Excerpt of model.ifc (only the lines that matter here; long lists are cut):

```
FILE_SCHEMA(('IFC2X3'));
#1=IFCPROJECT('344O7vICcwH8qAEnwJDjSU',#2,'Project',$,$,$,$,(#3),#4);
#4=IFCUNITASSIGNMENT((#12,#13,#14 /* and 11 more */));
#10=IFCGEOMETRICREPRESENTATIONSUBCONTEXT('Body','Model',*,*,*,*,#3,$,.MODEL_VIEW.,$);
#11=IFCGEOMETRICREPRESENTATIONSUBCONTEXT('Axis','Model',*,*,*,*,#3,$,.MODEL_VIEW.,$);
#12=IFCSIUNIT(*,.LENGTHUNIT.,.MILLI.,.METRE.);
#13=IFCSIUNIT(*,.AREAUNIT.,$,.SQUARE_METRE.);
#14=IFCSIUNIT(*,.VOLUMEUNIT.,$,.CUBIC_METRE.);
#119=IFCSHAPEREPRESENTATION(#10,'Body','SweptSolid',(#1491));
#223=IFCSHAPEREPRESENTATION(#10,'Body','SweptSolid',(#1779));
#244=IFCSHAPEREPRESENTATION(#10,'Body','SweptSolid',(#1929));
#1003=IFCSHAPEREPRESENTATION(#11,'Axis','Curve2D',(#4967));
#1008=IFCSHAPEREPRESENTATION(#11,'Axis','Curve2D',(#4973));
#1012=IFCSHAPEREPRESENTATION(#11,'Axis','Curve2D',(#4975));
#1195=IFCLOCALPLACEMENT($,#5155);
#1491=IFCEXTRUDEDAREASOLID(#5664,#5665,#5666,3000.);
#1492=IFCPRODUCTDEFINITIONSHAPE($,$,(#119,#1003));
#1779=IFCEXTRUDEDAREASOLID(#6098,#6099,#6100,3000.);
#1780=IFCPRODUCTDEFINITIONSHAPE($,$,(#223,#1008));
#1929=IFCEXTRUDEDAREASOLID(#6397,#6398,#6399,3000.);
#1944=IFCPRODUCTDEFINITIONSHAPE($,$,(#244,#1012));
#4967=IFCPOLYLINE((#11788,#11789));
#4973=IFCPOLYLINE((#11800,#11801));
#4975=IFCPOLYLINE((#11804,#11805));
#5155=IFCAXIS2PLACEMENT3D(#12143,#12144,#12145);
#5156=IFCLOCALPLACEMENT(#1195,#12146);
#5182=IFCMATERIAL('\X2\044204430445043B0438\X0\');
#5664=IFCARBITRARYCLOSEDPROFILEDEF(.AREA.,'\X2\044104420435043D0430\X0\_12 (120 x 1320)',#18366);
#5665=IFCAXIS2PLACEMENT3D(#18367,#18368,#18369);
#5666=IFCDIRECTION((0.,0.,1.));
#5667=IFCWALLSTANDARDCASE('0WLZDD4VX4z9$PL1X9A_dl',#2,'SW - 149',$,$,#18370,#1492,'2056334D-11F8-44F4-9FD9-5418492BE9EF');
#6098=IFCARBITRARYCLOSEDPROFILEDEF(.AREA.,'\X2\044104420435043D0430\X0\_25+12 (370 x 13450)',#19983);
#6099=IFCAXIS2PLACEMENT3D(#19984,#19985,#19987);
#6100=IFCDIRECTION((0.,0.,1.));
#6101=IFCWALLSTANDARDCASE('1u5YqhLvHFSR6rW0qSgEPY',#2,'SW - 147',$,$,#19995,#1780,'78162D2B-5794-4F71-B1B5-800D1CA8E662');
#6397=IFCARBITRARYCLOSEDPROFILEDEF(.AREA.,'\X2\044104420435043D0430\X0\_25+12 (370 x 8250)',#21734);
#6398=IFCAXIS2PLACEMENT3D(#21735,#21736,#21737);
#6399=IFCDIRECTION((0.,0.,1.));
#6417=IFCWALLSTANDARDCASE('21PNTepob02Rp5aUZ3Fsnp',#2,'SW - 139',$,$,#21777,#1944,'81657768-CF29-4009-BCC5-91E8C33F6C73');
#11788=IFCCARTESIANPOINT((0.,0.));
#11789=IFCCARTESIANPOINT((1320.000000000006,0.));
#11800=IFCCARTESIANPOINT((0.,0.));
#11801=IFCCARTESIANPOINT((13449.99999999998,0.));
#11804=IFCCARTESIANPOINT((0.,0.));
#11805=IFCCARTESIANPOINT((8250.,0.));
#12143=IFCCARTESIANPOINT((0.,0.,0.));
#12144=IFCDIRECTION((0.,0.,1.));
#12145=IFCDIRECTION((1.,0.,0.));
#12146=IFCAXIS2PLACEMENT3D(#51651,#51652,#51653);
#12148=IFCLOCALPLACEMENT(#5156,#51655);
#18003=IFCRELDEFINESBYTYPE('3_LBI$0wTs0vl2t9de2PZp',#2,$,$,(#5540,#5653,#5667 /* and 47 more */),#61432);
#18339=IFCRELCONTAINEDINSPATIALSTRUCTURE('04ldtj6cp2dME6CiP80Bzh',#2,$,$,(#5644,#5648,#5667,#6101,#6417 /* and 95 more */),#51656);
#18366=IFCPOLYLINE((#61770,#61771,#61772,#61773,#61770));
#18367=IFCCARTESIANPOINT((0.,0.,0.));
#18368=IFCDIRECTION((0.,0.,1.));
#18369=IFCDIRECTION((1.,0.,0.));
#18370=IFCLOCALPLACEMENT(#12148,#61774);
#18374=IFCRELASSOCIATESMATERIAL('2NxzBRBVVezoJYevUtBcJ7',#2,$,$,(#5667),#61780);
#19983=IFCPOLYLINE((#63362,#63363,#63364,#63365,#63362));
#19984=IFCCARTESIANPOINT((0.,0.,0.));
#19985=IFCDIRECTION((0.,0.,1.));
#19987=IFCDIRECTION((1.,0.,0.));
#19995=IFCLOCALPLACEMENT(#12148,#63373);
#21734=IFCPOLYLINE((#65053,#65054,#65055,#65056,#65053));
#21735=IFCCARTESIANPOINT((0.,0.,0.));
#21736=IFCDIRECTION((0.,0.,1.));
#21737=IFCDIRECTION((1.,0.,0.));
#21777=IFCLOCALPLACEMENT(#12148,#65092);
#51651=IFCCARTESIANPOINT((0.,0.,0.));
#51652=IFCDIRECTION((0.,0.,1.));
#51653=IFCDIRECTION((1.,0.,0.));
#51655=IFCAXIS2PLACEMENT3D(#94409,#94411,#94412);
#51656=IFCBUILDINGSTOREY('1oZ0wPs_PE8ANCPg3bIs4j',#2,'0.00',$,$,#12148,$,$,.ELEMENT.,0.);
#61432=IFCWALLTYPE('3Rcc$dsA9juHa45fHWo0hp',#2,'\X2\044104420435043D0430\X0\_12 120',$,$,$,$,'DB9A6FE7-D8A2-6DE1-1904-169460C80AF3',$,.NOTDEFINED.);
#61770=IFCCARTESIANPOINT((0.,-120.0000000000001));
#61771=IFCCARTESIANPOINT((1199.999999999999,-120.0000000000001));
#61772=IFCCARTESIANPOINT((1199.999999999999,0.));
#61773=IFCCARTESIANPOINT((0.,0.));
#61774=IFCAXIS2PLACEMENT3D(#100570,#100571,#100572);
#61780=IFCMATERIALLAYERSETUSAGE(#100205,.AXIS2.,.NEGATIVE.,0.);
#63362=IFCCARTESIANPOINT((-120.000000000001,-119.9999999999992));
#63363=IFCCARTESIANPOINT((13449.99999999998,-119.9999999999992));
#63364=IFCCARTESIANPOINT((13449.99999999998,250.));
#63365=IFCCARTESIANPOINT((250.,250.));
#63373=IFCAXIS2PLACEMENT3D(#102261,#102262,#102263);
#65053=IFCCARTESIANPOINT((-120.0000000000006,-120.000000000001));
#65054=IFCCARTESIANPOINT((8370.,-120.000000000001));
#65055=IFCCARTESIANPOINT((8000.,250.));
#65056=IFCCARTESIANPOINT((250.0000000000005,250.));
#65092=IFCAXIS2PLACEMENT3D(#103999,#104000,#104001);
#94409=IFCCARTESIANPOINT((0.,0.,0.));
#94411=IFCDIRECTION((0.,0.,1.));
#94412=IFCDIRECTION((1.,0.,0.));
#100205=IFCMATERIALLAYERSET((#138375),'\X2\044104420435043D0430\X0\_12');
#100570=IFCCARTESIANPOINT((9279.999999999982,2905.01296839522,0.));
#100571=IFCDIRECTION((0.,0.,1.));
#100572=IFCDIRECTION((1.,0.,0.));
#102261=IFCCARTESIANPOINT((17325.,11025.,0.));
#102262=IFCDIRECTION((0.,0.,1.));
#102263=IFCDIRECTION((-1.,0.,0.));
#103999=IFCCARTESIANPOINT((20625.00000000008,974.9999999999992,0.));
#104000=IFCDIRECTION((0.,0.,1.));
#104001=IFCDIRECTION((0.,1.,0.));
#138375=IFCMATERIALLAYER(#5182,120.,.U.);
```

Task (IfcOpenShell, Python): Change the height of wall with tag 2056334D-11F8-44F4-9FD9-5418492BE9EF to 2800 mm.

```python
import ifcopenshell
import ifcopenshell.geom
import ifcopenshell.util.representation
import ifcopenshell.util.shape
import ifcopenshell.util.unit

model = ifcopenshell.open("model.ifc")
unit_scale = ifcopenshell.util.unit.calculate_unit_scale(model)
settings = ifcopenshell.geom.settings()


def volume(element):
    """Net volume in cubic metres, openings subtracted."""
    shape = ifcopenshell.geom.create_shape(settings, element)
    return ifcopenshell.util.shape.get_volume(shape.geometry)


wall = model.by_guid("0WLZDD4VX4z9$PL1X9A_dl")
before = volume(wall)

body = ifcopenshell.util.representation.get_representation(wall, "Model", "Body")
solid = body.Items[0]
old_height = solid.Depth
solid.Depth = 2.8 / unit_scale
after = volume(wall)

print(f"height {old_height:g} -> {solid.Depth:g}, volume {before:.3f} -> {after:.3f} m3")

model.write("model-out.ifc")
```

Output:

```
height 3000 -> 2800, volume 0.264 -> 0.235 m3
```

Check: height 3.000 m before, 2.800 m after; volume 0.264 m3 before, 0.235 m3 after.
